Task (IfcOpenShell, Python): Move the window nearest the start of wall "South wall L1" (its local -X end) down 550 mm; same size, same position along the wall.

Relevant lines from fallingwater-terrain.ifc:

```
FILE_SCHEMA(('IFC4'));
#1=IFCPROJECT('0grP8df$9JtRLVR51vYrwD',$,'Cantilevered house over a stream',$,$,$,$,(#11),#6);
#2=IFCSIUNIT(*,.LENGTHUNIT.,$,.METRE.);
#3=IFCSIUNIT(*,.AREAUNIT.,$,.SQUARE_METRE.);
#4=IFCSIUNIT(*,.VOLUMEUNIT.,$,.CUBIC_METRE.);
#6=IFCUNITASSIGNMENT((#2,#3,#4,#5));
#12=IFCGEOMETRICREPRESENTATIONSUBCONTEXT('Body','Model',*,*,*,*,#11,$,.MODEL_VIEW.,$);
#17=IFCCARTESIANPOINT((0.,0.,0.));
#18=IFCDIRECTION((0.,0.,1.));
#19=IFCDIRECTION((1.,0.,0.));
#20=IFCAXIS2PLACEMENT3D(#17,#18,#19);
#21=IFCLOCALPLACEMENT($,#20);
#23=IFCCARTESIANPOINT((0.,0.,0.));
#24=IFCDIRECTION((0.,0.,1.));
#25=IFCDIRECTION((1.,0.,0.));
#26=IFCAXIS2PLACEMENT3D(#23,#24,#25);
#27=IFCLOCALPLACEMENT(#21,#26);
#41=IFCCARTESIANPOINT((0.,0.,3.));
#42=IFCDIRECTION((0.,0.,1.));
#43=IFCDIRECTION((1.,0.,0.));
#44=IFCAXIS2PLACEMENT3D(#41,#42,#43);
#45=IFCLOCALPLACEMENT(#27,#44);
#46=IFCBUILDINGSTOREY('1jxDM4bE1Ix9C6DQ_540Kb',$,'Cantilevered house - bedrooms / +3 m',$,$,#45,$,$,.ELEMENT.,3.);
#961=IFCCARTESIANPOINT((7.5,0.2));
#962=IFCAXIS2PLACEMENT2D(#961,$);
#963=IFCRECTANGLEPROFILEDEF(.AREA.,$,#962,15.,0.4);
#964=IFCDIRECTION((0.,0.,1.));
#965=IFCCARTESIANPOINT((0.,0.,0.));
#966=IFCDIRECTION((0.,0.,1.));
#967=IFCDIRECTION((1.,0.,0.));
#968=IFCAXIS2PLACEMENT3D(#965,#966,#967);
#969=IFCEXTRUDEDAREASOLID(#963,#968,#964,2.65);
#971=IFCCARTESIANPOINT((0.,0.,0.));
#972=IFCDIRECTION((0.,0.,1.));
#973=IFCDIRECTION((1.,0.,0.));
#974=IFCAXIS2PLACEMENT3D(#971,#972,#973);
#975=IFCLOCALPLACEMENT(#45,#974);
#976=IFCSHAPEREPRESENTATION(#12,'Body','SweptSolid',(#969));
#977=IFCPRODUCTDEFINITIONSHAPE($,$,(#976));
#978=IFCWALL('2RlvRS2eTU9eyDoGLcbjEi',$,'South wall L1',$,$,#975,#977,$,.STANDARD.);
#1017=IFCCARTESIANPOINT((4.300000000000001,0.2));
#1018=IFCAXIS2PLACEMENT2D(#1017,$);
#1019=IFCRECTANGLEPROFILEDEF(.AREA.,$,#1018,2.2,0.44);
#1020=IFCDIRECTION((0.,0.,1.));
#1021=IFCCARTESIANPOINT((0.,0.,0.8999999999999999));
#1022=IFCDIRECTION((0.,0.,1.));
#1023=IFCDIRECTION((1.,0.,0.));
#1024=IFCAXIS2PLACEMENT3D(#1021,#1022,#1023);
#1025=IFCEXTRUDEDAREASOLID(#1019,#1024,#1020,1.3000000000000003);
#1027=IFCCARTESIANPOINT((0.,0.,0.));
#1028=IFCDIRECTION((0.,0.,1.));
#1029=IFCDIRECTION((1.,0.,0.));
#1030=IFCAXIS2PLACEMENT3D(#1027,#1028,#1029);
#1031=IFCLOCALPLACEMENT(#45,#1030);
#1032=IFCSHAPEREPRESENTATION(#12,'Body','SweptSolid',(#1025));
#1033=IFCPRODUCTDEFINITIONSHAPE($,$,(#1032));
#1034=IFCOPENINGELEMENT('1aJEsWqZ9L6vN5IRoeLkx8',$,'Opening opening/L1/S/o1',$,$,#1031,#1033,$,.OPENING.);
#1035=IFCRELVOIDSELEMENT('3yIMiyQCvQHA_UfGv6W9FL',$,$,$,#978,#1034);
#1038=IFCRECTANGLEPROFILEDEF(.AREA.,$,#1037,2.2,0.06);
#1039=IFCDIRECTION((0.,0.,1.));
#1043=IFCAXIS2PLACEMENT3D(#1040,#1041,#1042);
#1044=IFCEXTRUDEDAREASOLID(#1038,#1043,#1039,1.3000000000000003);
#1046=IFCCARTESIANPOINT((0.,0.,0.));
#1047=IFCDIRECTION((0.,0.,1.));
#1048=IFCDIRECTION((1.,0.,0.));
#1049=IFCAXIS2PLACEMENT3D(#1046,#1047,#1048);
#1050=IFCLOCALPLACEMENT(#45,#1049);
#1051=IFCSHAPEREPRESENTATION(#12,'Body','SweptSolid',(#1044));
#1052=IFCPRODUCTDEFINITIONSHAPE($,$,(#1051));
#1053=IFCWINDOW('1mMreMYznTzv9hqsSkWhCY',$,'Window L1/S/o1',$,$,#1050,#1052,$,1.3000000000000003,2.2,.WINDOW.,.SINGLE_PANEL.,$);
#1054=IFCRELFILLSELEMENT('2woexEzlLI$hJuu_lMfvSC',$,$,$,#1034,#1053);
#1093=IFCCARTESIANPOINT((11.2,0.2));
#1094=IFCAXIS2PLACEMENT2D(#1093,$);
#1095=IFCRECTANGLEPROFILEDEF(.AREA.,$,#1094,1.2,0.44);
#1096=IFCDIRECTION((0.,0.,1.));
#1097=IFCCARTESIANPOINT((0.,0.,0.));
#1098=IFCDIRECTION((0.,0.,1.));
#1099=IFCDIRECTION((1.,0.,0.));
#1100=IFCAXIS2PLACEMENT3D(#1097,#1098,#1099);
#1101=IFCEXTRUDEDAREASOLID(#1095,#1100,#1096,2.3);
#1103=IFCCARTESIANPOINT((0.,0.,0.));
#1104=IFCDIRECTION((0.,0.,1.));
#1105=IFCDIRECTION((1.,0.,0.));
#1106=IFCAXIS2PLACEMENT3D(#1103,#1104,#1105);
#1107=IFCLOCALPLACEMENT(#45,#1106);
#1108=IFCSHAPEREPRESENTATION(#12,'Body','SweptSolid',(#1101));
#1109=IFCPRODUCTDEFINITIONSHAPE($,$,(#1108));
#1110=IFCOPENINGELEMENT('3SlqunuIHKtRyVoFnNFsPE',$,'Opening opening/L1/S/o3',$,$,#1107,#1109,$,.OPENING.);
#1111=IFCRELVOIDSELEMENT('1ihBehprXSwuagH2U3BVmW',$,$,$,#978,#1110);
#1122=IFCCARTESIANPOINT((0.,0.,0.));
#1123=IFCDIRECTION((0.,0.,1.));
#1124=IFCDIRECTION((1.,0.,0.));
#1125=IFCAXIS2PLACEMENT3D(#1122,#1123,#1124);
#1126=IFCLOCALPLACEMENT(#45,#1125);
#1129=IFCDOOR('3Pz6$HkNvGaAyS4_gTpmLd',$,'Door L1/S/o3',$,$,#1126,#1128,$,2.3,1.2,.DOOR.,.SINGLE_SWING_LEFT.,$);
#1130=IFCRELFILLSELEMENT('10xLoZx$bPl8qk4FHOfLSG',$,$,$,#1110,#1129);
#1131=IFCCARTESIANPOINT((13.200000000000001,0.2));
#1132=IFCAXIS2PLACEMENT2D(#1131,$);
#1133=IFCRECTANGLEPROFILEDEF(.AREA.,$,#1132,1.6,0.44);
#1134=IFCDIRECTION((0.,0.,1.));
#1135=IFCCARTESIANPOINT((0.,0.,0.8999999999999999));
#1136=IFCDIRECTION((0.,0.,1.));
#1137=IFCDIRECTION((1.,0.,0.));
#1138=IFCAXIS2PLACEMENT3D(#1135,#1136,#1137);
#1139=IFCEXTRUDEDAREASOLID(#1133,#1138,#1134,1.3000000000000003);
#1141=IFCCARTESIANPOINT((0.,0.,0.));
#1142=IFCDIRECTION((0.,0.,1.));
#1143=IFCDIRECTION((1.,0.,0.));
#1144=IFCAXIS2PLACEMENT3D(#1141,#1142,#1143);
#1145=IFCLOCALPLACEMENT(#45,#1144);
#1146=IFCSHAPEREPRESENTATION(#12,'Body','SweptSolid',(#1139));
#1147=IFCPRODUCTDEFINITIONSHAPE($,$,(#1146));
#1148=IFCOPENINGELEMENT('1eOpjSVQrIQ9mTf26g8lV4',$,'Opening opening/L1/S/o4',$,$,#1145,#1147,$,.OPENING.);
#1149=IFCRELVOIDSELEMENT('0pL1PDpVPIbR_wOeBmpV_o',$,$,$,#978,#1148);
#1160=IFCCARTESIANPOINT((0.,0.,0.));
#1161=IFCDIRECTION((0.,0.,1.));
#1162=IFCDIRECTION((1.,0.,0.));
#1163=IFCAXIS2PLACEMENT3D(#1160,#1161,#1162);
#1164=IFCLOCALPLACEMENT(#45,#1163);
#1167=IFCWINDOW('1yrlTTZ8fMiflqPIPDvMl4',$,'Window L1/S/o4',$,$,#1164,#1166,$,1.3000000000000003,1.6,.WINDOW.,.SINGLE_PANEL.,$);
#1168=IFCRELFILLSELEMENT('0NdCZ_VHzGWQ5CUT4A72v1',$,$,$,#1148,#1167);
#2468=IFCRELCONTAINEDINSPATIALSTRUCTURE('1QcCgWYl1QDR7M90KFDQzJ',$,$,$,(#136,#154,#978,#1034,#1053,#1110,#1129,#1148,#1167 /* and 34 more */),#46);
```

```python
import numpy as np
import ifcopenshell
import ifcopenshell.api.geometry
import ifcopenshell.util.placement
import ifcopenshell.util.unit

model = ifcopenshell.open("fallingwater-terrain.ifc")
unit_scale = ifcopenshell.util.unit.calculate_unit_scale(model)

window = model.by_guid("1mMreMYznTzv9hqsSkWhCY")
opening = window.FillsVoids[0].RelatingOpeningElement
dz = -0.55 / unit_scale

shift = np.array([0.0, 0.0, dz])
# The window is not placed relative to its opening, so move both.
for product in (opening, window):
    matrix = ifcopenshell.util.placement.get_local_placement(product.ObjectPlacement)
    matrix[:3, 3] += shift
    ifcopenshell.api.geometry.edit_object_placement(model, product=product, matrix=matrix, is_si=False)

print(f"moved by {dz * unit_scale:+.3f} m")

model.write("fallingwater-terrain_v2.ifc")
```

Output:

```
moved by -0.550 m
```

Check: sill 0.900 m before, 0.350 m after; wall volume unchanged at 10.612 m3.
